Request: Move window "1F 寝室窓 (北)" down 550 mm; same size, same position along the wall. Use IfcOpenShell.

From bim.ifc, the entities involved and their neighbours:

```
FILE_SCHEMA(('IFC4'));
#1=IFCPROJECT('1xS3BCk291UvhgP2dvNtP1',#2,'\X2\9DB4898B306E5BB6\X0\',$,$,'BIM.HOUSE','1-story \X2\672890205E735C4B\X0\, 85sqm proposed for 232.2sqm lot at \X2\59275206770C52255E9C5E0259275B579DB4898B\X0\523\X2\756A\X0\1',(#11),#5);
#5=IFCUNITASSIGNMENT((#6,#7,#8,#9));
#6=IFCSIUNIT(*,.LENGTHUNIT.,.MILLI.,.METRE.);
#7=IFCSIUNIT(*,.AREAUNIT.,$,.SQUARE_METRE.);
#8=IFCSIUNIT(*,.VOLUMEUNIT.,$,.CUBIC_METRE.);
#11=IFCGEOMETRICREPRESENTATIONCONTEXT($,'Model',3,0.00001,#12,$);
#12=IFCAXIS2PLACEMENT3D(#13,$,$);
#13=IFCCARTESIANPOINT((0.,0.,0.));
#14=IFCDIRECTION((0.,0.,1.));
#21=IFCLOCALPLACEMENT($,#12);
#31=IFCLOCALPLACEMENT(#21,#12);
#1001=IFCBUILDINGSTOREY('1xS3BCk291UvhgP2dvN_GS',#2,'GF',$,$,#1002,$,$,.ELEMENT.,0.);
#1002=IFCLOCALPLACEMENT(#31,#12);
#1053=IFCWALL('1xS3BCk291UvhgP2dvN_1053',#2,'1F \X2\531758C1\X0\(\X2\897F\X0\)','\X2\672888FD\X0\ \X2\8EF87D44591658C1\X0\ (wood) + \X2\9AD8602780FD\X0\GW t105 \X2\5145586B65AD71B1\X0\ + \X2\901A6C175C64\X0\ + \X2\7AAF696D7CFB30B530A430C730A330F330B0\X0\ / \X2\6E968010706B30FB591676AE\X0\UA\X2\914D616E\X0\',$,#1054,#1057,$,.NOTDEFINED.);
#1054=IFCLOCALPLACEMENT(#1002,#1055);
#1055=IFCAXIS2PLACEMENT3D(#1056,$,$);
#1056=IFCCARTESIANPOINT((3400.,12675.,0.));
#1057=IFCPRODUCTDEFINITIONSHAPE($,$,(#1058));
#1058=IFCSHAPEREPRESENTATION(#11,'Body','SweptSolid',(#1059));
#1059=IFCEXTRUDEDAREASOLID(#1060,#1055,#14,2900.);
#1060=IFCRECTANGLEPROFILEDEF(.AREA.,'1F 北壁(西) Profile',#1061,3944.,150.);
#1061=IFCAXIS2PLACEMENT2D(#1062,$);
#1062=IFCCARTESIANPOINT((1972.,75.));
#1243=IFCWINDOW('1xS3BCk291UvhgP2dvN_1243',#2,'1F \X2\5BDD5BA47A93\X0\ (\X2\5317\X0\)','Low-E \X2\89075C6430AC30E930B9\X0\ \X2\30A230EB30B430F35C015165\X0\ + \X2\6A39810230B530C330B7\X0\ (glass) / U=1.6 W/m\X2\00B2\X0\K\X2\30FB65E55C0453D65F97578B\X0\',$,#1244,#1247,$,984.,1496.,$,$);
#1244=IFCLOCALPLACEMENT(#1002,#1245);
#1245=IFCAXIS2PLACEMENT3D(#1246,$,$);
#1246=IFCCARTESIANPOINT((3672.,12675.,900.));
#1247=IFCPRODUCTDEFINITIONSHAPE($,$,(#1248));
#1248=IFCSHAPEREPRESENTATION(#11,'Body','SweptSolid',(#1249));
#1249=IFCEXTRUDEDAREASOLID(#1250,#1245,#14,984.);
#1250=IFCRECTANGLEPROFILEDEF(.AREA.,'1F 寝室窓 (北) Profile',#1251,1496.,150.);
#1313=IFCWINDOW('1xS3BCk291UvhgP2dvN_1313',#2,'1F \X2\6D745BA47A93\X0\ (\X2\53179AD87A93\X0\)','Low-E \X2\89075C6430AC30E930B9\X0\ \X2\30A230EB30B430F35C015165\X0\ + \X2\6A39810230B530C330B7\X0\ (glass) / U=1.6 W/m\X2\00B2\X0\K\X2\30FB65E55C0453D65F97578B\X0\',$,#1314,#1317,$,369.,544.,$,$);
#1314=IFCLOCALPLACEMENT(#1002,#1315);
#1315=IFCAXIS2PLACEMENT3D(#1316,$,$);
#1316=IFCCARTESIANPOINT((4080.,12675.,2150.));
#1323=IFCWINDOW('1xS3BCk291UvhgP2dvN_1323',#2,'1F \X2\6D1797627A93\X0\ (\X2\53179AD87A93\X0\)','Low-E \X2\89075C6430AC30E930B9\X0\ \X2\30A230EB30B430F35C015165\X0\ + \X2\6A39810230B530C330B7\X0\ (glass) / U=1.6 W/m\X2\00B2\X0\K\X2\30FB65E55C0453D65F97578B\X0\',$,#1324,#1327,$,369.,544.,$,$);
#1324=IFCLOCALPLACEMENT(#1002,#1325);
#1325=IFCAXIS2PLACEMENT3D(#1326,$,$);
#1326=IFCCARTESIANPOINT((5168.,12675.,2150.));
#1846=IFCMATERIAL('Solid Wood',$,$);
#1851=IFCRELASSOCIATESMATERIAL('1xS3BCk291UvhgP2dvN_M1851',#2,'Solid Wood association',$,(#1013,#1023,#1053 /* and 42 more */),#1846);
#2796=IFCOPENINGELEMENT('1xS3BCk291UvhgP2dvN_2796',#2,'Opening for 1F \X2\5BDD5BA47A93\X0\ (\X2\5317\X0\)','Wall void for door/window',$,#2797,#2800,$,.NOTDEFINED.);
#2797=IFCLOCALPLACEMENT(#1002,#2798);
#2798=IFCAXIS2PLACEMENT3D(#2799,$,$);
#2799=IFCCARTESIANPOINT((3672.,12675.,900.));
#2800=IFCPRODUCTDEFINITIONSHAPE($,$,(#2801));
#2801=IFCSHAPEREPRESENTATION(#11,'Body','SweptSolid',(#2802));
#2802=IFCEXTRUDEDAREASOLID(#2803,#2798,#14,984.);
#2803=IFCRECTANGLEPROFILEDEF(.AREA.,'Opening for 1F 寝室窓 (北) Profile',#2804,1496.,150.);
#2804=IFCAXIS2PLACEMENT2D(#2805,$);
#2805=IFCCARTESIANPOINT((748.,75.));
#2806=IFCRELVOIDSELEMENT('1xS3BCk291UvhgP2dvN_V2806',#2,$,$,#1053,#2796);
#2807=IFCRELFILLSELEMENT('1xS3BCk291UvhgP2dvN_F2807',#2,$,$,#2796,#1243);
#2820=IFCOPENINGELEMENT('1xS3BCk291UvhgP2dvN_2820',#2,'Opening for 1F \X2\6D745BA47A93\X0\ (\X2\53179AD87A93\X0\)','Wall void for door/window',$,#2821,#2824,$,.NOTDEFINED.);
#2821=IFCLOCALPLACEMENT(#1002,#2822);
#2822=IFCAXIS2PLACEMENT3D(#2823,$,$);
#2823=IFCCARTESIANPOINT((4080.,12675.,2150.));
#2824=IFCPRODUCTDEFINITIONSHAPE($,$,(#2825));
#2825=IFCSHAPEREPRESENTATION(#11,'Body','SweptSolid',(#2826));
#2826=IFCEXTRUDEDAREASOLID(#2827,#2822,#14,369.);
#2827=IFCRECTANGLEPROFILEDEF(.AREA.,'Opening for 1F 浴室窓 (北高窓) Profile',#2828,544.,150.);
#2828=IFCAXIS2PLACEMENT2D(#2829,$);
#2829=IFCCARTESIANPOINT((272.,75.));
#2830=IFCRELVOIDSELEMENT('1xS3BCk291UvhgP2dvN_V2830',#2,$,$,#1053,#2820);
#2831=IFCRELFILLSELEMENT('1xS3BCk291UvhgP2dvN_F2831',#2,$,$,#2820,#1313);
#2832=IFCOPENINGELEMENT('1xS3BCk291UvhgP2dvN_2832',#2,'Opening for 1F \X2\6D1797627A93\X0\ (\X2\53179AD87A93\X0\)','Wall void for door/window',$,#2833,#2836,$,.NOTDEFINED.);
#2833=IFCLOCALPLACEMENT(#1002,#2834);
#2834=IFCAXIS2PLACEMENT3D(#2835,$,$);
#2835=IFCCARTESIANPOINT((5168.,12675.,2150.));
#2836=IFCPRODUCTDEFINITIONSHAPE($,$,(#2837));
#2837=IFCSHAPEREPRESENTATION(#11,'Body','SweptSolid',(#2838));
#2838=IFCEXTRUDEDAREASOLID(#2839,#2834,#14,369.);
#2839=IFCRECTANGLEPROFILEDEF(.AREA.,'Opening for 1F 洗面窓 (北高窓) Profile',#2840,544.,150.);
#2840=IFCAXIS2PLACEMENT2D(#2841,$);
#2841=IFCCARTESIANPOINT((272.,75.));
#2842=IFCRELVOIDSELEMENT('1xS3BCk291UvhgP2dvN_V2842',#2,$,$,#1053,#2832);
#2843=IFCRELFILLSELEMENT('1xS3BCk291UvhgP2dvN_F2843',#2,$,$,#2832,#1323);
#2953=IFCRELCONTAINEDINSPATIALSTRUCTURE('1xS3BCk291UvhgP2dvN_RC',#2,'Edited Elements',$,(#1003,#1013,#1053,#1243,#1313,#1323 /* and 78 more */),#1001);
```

```python
import numpy as np
import ifcopenshell
import ifcopenshell.api.geometry
import ifcopenshell.util.placement
import ifcopenshell.util.unit

model = ifcopenshell.open("bim.ifc")
unit_scale = ifcopenshell.util.unit.calculate_unit_scale(model)

window = model.by_id(1243)
opening = window.FillsVoids[0].RelatingOpeningElement
dz = -0.55 / unit_scale

shift = np.array([0.0, 0.0, dz])
# The window is not placed relative to its opening, so move both.
for product in (opening, window):
    matrix = ifcopenshell.util.placement.get_local_placement(product.ObjectPlacement)
    matrix[:3, 3] += shift
    ifcopenshell.api.geometry.edit_object_placement(model, product=product, matrix=matrix, is_si=False)

print(f"moved by {dz * unit_scale:+.3f} m")

model.write("bim_v2.ifc")
```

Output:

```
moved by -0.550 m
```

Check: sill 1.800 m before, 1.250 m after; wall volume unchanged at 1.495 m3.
